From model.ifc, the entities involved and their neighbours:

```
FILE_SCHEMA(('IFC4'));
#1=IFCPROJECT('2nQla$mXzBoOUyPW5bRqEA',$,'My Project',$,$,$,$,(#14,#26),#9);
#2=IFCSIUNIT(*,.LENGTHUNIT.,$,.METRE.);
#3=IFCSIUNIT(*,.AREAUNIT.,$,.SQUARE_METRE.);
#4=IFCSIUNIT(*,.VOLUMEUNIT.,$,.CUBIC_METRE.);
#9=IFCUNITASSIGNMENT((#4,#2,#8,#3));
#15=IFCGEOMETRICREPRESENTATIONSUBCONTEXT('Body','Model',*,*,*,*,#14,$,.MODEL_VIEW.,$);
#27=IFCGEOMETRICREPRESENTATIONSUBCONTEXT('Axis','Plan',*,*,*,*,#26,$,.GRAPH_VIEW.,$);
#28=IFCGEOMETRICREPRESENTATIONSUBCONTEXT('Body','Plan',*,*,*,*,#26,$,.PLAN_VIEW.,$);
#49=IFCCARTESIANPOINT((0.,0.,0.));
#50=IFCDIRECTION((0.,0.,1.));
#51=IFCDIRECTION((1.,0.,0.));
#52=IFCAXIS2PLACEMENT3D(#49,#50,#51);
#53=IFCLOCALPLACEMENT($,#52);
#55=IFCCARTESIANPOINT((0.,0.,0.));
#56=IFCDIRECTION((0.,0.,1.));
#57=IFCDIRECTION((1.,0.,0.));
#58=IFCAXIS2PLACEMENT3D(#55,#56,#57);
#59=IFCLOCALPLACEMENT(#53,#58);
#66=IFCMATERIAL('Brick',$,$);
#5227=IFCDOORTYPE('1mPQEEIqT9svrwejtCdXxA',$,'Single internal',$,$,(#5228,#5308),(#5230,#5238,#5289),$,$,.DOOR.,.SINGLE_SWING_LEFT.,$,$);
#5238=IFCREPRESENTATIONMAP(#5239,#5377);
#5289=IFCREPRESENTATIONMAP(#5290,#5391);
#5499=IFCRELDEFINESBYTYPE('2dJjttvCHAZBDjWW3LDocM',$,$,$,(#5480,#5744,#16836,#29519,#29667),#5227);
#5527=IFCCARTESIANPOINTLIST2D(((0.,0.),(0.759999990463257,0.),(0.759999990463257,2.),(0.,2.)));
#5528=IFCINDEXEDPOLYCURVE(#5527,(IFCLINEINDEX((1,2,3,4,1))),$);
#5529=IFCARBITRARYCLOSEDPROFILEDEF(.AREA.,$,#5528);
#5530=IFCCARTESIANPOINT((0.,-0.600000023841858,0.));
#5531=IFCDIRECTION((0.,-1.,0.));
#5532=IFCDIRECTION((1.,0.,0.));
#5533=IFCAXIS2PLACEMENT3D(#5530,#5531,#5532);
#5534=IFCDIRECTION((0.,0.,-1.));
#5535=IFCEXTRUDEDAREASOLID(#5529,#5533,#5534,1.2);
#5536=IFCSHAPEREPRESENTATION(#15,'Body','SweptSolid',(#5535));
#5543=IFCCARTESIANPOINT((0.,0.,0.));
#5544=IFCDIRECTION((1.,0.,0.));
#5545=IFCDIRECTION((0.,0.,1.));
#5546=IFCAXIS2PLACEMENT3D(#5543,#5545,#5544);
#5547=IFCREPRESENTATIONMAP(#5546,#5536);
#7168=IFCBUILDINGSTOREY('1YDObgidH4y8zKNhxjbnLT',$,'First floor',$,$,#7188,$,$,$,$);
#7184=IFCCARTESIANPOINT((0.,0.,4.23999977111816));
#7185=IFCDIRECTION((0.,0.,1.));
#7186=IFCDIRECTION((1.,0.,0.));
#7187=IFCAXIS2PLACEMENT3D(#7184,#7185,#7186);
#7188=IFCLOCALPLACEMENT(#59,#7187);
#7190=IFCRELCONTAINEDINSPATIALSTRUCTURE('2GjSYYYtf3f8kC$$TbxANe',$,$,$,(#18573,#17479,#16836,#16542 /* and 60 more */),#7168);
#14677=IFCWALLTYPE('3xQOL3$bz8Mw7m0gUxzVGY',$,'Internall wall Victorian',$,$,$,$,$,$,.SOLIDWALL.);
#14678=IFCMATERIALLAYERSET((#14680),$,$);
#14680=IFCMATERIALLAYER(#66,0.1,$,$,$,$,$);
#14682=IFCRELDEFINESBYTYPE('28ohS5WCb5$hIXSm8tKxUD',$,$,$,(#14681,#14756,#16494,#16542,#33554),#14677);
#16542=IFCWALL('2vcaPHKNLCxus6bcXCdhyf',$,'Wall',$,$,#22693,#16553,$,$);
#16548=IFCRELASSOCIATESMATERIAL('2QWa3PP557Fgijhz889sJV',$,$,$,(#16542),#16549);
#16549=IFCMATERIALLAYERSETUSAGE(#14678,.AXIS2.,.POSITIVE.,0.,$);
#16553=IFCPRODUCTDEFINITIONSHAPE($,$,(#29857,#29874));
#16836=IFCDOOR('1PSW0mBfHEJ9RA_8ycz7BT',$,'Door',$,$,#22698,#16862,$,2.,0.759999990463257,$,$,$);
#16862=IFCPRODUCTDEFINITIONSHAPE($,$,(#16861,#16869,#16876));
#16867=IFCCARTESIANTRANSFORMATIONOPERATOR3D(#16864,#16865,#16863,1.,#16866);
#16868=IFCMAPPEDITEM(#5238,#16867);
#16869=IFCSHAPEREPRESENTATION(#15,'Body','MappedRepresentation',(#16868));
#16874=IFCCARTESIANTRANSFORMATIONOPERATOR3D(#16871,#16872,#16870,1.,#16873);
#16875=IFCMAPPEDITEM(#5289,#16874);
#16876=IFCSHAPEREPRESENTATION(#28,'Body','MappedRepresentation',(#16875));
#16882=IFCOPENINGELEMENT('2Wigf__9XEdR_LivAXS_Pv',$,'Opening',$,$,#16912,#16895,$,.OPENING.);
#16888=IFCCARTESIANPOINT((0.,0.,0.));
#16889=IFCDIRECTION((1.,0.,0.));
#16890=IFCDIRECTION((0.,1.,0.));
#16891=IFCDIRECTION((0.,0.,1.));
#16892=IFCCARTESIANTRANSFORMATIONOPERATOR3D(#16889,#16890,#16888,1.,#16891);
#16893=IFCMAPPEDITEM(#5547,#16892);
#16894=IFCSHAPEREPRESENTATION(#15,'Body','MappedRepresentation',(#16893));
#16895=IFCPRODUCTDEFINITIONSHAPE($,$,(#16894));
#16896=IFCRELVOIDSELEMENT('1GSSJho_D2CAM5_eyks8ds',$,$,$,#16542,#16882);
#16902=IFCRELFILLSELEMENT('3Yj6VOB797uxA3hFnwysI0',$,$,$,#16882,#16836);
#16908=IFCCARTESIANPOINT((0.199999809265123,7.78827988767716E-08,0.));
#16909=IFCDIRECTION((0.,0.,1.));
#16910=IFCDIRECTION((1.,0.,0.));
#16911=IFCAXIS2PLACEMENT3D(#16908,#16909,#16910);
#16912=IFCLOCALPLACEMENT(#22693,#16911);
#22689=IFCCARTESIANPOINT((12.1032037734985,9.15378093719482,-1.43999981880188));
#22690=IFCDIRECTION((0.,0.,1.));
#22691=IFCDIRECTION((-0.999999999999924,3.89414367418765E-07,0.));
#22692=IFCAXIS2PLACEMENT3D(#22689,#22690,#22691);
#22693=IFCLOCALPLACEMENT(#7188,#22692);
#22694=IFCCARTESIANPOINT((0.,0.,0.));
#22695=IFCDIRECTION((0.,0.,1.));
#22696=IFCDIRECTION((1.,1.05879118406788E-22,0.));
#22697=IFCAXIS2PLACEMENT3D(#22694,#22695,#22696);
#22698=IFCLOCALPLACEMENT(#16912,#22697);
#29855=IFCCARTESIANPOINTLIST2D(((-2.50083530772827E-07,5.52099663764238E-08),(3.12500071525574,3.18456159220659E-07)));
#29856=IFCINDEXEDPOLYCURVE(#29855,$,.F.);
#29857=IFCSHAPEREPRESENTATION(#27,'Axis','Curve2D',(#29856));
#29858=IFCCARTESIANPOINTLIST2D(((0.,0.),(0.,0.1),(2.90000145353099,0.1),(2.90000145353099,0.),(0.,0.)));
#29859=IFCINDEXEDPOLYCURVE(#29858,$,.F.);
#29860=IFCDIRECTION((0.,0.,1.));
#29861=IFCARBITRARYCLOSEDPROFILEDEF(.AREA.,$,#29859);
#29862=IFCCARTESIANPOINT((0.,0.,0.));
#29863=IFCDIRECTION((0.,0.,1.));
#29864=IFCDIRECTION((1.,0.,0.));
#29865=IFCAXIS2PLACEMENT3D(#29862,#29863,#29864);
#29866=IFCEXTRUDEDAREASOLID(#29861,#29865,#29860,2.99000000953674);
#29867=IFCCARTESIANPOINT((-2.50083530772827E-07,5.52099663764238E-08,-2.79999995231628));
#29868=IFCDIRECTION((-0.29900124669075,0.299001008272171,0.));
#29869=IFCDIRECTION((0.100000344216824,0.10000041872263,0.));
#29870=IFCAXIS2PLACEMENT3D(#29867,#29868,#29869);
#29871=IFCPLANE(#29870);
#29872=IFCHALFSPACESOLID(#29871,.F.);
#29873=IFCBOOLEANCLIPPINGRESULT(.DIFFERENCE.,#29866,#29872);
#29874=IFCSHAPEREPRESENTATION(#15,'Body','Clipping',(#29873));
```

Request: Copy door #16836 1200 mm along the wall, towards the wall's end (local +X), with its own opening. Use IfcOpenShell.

```python
import ifcopenshell
import ifcopenshell.api.feature
import ifcopenshell.api.geometry
import ifcopenshell.api.root
import ifcopenshell.geom
import ifcopenshell.util.element
import ifcopenshell.util.placement
import ifcopenshell.util.shape
import ifcopenshell.util.unit

model = ifcopenshell.open("model.ifc")
unit_scale = ifcopenshell.util.unit.calculate_unit_scale(model)
settings = ifcopenshell.geom.settings()


def volume(element):
    """Net volume in cubic metres, openings subtracted."""
    shape = ifcopenshell.geom.create_shape(settings, element)
    return ifcopenshell.util.shape.get_volume(shape.geometry)


door = model.by_id(16836)
opening = door.FillsVoids[0].RelatingOpeningElement
wall = opening.VoidsElements[0].RelatingBuildingElement
before = volume(wall)
shift = ifcopenshell.util.placement.get_local_placement(wall.ObjectPlacement)[:3, 0] * 1.2 / unit_scale

# copy_class copies the void relationship, type, container and properties, but no geometry.
new_opening = ifcopenshell.api.root.copy_class(model, product=opening)
new_opening.Representation = ifcopenshell.util.element.copy_deep(
    model, opening.Representation, exclude=["IfcGeometricRepresentationContext", "IfcRepresentationMap"]
)
new_door = ifcopenshell.api.root.copy_class(model, product=door)
new_door.Representation = ifcopenshell.util.element.copy_deep(
    model, door.Representation, exclude=["IfcGeometricRepresentationContext", "IfcRepresentationMap"]
)
ifcopenshell.api.feature.add_filling(model, opening=new_opening, element=new_door)

for old, new in ((opening, new_opening), (door, new_door)):
    matrix = ifcopenshell.util.placement.get_local_placement(old.ObjectPlacement)
    matrix[:3, 3] += shift
    ifcopenshell.api.geometry.edit_object_placement(model, product=new, matrix=matrix, is_si=False)

after = volume(wall)

print(f"wall volume {before:.3f} -> {after:.3f} m3")

model.write("model_updated.ifc")
```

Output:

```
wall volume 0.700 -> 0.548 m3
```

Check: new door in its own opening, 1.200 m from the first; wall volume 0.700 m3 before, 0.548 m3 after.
